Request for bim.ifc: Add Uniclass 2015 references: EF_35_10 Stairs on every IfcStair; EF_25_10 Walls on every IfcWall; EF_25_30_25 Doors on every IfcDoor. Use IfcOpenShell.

First a look at what the model holds.

```python
import ifcopenshell

model = ifcopenshell.open("bim.ifc")
print(model.schema)
print("classifications:", [c.Name for c in model.by_type("IfcClassification")])
for ifc_class in ("IfcDoor", "IfcRoof", "IfcStair", "IfcWall", "IfcWindow"):
    print(ifc_class, len(model.by_type(ifc_class)))
```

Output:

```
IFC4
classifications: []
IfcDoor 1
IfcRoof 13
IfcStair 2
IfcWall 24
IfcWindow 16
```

```python
import ifcopenshell
import ifcopenshell.api.classification

model = ifcopenshell.open("bim.ifc")

system = ifcopenshell.api.classification.add_classification(model, classification="Uniclass 2015")

codes = {
    "IfcStair": ("EF_35_10", "Stairs"),
    "IfcWall": ("EF_25_10", "Walls"),
    "IfcDoor": ("EF_25_30_25", "Doors"),
}
for ifc_class, (code, name) in codes.items():
    products = model.by_type(ifc_class)
    ifcopenshell.api.classification.add_reference(
        model, products=products, classification=system, identification=code, name=name
    )
    print(code, len(products))

model.write("bim_v2.ifc")
```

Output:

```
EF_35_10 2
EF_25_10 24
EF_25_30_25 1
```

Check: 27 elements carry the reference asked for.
